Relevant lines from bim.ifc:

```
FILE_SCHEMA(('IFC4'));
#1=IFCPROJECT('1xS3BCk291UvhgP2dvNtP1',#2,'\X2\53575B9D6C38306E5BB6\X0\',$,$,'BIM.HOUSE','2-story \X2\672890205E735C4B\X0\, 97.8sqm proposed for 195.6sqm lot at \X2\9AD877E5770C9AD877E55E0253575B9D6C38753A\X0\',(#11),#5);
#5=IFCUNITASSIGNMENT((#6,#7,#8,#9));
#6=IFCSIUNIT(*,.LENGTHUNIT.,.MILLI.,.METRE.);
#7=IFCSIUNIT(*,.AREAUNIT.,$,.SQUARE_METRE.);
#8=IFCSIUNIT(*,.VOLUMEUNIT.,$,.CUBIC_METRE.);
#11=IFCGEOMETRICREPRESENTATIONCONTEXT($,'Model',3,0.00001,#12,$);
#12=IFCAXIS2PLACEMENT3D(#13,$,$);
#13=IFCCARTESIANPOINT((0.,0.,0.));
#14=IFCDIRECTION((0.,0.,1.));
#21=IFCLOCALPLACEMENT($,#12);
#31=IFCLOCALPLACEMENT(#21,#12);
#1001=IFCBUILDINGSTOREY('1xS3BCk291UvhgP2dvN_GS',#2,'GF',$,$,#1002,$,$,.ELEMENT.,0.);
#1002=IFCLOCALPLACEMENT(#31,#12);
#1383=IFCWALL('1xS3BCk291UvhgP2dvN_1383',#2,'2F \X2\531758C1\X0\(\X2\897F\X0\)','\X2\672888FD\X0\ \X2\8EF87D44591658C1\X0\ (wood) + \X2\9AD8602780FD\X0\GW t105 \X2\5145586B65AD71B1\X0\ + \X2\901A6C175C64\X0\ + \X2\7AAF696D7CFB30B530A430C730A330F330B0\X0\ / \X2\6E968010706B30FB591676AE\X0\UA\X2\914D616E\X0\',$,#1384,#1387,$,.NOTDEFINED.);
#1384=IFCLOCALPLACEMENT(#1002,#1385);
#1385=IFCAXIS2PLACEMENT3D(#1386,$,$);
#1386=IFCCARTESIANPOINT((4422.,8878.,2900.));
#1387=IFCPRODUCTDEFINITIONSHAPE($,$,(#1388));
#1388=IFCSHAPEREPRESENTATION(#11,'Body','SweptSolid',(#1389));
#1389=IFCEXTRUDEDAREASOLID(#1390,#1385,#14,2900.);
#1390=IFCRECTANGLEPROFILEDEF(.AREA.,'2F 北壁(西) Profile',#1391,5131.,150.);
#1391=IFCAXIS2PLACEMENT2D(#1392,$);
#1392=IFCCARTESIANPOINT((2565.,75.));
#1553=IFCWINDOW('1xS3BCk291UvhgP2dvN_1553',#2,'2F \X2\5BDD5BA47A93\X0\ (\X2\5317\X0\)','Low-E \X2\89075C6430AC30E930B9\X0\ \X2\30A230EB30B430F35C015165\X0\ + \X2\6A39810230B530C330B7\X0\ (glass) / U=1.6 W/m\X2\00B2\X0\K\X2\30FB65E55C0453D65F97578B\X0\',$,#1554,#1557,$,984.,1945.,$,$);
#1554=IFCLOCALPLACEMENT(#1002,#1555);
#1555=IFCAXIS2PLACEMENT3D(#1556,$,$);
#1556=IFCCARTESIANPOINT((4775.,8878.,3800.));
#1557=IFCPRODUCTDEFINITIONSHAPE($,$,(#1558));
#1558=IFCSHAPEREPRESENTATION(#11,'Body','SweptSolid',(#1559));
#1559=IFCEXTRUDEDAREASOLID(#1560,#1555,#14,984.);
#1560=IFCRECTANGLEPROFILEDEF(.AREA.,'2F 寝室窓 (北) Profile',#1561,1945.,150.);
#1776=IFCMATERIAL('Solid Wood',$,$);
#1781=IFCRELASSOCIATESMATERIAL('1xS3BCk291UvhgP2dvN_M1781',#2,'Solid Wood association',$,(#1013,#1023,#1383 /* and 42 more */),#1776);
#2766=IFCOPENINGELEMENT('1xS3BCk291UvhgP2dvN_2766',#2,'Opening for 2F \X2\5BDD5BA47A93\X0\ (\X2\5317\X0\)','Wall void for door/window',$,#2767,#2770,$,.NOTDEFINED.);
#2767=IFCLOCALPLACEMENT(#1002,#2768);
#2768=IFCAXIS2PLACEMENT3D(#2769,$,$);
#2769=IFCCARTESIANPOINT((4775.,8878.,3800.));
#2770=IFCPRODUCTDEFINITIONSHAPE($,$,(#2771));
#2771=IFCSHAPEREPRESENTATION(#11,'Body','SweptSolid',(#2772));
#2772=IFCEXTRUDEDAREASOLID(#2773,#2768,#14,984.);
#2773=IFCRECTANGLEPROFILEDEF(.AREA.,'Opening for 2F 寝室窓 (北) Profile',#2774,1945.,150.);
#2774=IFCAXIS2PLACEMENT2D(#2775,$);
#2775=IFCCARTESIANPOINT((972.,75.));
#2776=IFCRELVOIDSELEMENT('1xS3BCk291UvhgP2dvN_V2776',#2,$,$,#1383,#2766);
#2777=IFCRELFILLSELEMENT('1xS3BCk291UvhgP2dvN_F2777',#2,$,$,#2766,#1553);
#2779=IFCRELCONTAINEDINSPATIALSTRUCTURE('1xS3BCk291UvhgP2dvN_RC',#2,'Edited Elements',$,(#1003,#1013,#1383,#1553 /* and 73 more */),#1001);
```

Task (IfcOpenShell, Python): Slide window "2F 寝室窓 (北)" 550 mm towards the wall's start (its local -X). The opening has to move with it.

```python
import ifcopenshell
import ifcopenshell.api.geometry
import ifcopenshell.util.placement
import ifcopenshell.util.unit

model = ifcopenshell.open("bim.ifc")
unit_scale = ifcopenshell.util.unit.calculate_unit_scale(model)

window = model.by_guid("1xS3BCk291UvhgP2dvN_1553")
opening = window.FillsVoids[0].RelatingOpeningElement
wall = opening.VoidsElements[0].RelatingBuildingElement

wall_matrix = ifcopenshell.util.placement.get_local_placement(wall.ObjectPlacement)
shift = wall_matrix[:3, 0] * -0.55 / unit_scale
before = ifcopenshell.util.placement.get_local_placement(window.ObjectPlacement)[:3, 3].copy()

# The window is not placed relative to its opening, so move both.
for product in (opening, window):
    matrix = ifcopenshell.util.placement.get_local_placement(product.ObjectPlacement)
    matrix[:3, 3] += shift
    ifcopenshell.api.geometry.edit_object_placement(model, product=product, matrix=matrix, is_si=False)

after = ifcopenshell.util.placement.get_local_placement(window.ObjectPlacement)[:3, 3]
print("window moved by", (after - before).round(3) + 0.0)

model.write("bim_edited.ifc")
```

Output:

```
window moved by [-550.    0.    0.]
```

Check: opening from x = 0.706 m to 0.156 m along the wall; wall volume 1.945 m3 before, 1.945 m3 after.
